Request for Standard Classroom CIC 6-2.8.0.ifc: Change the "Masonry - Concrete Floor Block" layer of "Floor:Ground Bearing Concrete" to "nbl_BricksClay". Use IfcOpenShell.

First a look at what the model holds.

```python
import ifcopenshell
import ifcopenshell.util.element

model = ifcopenshell.open("Standard Classroom CIC 6-2.8.0.ifc")
print(model.schema)
for layer_set in model.by_type("IfcMaterialLayerSet"):
    if layer_set.LayerSetName == "Floor:Ground Bearing Concrete":
        for layer in layer_set.MaterialLayers:
            print(layer.id(), layer.Material and layer.Material.Name, layer.LayerThickness, sep=" | ")
        print(len(ifcopenshell.util.element.get_elements_by_material(model, layer_set)), "elements and types use it")
print(sorted(m.Name for m in model.by_type("IfcMaterial") if m.Name)[:60])
```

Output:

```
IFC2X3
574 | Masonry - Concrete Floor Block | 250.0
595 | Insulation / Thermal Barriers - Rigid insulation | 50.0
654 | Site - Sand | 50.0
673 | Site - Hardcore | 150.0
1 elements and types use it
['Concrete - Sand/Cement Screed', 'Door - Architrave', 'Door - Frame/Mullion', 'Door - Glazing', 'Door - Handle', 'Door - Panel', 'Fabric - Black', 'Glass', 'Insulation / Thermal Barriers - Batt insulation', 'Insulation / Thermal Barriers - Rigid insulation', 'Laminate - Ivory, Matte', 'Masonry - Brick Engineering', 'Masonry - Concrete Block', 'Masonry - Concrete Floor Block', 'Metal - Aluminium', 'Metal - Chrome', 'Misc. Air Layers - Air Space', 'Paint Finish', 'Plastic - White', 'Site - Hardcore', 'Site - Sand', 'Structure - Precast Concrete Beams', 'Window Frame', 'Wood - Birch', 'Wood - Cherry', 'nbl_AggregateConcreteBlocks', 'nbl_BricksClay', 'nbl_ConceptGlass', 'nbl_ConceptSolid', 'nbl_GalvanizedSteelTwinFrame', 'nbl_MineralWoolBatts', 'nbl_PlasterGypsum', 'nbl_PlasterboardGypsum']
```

```python
import ifcopenshell
import ifcopenshell.api.material

model = ifcopenshell.open("Standard Classroom CIC 6-2.8.0.ifc")

layer_set = next(s for s in model.by_type("IfcMaterialLayerSet") if s.LayerSetName == "Floor:Ground Bearing Concrete")
layer = next(l for l in layer_set.MaterialLayers if l.Material and l.Material.Name == "Masonry - Concrete Floor Block")
material = next(m for m in model.by_type("IfcMaterial") if m.Name == "nbl_BricksClay")

# Point this one layer at the other material; renaming the old one would change it everywhere.
ifcopenshell.api.material.edit_layer(model, layer=layer, attributes={}, material=material)

print([l.Material.Name if l.Material else None for l in layer_set.MaterialLayers])

model.write("Standard Classroom CIC 6-2.8.0_v2.ifc")
```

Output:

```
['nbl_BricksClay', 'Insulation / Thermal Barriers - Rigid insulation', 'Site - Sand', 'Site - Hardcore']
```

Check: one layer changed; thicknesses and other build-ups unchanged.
